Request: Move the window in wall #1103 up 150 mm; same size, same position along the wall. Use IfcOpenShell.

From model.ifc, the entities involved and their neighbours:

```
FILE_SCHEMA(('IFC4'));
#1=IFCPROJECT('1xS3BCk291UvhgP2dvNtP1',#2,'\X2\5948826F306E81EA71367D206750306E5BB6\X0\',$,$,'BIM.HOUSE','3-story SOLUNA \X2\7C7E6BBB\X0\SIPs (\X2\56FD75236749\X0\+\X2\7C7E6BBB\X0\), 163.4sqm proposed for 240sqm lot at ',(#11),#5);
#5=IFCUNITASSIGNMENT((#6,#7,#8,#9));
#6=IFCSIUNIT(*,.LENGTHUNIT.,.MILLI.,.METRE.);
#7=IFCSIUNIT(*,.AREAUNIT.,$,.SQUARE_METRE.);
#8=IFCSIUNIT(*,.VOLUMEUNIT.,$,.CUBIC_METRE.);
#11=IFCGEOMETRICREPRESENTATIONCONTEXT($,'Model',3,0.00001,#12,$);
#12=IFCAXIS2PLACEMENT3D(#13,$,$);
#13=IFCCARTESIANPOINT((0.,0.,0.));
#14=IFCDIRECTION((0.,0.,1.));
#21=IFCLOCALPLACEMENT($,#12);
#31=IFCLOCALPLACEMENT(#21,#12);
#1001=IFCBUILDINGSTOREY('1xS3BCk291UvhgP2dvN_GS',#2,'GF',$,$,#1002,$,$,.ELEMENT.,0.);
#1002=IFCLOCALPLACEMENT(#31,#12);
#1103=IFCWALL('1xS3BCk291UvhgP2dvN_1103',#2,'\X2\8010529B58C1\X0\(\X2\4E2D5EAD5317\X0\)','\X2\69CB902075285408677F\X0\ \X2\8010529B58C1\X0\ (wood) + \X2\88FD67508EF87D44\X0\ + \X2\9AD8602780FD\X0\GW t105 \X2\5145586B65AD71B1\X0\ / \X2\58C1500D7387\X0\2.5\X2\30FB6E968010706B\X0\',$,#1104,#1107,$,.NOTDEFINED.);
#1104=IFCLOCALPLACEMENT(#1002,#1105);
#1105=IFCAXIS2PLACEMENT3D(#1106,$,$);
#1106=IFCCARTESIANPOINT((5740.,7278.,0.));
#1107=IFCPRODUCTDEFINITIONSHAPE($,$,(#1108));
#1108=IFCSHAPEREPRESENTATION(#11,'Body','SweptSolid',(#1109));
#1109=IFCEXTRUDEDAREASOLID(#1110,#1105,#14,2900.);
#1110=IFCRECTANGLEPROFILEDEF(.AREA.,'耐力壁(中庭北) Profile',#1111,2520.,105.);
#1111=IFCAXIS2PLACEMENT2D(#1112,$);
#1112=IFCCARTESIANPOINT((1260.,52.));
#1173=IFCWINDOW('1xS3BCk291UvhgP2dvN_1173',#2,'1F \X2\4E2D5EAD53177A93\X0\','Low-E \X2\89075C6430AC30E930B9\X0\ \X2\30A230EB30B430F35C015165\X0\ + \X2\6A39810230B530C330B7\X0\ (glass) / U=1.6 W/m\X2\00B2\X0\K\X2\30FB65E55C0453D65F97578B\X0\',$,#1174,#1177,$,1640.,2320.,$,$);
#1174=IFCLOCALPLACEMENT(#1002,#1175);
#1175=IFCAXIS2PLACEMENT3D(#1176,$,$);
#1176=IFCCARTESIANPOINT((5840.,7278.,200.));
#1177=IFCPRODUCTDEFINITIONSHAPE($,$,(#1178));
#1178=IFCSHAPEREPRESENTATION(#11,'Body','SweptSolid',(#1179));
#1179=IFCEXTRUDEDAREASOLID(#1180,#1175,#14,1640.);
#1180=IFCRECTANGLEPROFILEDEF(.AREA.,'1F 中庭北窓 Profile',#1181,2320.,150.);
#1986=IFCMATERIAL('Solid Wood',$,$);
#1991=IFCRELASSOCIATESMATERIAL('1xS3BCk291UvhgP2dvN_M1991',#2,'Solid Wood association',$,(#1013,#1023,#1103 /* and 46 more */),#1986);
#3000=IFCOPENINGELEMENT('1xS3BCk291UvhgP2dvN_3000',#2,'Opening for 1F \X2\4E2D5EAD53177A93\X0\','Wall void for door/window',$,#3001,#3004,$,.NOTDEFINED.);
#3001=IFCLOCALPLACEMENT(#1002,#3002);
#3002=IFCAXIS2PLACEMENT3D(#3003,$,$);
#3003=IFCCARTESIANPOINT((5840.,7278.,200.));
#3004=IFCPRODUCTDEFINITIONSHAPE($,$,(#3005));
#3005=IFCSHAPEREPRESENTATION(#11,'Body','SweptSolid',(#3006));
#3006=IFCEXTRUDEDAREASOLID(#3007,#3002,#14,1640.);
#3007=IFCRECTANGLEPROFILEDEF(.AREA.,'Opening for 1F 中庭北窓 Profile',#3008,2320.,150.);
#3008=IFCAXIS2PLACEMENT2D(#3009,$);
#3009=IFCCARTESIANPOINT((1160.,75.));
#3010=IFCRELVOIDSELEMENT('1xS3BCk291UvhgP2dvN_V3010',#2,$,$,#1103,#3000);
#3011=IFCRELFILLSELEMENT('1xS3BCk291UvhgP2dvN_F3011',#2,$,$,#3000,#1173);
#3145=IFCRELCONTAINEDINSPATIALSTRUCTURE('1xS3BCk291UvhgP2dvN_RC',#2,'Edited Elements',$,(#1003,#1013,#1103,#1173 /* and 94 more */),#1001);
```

```python
import numpy as np
import ifcopenshell
import ifcopenshell.api.geometry
import ifcopenshell.util.placement
import ifcopenshell.util.unit

model = ifcopenshell.open("model.ifc")
unit_scale = ifcopenshell.util.unit.calculate_unit_scale(model)

window = model.by_guid("1xS3BCk291UvhgP2dvN_1173")
opening = window.FillsVoids[0].RelatingOpeningElement
dz = 0.15 / unit_scale

shift = np.array([0.0, 0.0, dz])
# The window is not placed relative to its opening, so move both.
for product in (opening, window):
    matrix = ifcopenshell.util.placement.get_local_placement(product.ObjectPlacement)
    matrix[:3, 3] += shift
    ifcopenshell.api.geometry.edit_object_placement(model, product=product, matrix=matrix, is_si=False)

print(f"moved by {dz * unit_scale:+.3f} m")

model.write("model_v2.ifc")
```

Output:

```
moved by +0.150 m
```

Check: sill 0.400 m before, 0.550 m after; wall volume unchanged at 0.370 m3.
